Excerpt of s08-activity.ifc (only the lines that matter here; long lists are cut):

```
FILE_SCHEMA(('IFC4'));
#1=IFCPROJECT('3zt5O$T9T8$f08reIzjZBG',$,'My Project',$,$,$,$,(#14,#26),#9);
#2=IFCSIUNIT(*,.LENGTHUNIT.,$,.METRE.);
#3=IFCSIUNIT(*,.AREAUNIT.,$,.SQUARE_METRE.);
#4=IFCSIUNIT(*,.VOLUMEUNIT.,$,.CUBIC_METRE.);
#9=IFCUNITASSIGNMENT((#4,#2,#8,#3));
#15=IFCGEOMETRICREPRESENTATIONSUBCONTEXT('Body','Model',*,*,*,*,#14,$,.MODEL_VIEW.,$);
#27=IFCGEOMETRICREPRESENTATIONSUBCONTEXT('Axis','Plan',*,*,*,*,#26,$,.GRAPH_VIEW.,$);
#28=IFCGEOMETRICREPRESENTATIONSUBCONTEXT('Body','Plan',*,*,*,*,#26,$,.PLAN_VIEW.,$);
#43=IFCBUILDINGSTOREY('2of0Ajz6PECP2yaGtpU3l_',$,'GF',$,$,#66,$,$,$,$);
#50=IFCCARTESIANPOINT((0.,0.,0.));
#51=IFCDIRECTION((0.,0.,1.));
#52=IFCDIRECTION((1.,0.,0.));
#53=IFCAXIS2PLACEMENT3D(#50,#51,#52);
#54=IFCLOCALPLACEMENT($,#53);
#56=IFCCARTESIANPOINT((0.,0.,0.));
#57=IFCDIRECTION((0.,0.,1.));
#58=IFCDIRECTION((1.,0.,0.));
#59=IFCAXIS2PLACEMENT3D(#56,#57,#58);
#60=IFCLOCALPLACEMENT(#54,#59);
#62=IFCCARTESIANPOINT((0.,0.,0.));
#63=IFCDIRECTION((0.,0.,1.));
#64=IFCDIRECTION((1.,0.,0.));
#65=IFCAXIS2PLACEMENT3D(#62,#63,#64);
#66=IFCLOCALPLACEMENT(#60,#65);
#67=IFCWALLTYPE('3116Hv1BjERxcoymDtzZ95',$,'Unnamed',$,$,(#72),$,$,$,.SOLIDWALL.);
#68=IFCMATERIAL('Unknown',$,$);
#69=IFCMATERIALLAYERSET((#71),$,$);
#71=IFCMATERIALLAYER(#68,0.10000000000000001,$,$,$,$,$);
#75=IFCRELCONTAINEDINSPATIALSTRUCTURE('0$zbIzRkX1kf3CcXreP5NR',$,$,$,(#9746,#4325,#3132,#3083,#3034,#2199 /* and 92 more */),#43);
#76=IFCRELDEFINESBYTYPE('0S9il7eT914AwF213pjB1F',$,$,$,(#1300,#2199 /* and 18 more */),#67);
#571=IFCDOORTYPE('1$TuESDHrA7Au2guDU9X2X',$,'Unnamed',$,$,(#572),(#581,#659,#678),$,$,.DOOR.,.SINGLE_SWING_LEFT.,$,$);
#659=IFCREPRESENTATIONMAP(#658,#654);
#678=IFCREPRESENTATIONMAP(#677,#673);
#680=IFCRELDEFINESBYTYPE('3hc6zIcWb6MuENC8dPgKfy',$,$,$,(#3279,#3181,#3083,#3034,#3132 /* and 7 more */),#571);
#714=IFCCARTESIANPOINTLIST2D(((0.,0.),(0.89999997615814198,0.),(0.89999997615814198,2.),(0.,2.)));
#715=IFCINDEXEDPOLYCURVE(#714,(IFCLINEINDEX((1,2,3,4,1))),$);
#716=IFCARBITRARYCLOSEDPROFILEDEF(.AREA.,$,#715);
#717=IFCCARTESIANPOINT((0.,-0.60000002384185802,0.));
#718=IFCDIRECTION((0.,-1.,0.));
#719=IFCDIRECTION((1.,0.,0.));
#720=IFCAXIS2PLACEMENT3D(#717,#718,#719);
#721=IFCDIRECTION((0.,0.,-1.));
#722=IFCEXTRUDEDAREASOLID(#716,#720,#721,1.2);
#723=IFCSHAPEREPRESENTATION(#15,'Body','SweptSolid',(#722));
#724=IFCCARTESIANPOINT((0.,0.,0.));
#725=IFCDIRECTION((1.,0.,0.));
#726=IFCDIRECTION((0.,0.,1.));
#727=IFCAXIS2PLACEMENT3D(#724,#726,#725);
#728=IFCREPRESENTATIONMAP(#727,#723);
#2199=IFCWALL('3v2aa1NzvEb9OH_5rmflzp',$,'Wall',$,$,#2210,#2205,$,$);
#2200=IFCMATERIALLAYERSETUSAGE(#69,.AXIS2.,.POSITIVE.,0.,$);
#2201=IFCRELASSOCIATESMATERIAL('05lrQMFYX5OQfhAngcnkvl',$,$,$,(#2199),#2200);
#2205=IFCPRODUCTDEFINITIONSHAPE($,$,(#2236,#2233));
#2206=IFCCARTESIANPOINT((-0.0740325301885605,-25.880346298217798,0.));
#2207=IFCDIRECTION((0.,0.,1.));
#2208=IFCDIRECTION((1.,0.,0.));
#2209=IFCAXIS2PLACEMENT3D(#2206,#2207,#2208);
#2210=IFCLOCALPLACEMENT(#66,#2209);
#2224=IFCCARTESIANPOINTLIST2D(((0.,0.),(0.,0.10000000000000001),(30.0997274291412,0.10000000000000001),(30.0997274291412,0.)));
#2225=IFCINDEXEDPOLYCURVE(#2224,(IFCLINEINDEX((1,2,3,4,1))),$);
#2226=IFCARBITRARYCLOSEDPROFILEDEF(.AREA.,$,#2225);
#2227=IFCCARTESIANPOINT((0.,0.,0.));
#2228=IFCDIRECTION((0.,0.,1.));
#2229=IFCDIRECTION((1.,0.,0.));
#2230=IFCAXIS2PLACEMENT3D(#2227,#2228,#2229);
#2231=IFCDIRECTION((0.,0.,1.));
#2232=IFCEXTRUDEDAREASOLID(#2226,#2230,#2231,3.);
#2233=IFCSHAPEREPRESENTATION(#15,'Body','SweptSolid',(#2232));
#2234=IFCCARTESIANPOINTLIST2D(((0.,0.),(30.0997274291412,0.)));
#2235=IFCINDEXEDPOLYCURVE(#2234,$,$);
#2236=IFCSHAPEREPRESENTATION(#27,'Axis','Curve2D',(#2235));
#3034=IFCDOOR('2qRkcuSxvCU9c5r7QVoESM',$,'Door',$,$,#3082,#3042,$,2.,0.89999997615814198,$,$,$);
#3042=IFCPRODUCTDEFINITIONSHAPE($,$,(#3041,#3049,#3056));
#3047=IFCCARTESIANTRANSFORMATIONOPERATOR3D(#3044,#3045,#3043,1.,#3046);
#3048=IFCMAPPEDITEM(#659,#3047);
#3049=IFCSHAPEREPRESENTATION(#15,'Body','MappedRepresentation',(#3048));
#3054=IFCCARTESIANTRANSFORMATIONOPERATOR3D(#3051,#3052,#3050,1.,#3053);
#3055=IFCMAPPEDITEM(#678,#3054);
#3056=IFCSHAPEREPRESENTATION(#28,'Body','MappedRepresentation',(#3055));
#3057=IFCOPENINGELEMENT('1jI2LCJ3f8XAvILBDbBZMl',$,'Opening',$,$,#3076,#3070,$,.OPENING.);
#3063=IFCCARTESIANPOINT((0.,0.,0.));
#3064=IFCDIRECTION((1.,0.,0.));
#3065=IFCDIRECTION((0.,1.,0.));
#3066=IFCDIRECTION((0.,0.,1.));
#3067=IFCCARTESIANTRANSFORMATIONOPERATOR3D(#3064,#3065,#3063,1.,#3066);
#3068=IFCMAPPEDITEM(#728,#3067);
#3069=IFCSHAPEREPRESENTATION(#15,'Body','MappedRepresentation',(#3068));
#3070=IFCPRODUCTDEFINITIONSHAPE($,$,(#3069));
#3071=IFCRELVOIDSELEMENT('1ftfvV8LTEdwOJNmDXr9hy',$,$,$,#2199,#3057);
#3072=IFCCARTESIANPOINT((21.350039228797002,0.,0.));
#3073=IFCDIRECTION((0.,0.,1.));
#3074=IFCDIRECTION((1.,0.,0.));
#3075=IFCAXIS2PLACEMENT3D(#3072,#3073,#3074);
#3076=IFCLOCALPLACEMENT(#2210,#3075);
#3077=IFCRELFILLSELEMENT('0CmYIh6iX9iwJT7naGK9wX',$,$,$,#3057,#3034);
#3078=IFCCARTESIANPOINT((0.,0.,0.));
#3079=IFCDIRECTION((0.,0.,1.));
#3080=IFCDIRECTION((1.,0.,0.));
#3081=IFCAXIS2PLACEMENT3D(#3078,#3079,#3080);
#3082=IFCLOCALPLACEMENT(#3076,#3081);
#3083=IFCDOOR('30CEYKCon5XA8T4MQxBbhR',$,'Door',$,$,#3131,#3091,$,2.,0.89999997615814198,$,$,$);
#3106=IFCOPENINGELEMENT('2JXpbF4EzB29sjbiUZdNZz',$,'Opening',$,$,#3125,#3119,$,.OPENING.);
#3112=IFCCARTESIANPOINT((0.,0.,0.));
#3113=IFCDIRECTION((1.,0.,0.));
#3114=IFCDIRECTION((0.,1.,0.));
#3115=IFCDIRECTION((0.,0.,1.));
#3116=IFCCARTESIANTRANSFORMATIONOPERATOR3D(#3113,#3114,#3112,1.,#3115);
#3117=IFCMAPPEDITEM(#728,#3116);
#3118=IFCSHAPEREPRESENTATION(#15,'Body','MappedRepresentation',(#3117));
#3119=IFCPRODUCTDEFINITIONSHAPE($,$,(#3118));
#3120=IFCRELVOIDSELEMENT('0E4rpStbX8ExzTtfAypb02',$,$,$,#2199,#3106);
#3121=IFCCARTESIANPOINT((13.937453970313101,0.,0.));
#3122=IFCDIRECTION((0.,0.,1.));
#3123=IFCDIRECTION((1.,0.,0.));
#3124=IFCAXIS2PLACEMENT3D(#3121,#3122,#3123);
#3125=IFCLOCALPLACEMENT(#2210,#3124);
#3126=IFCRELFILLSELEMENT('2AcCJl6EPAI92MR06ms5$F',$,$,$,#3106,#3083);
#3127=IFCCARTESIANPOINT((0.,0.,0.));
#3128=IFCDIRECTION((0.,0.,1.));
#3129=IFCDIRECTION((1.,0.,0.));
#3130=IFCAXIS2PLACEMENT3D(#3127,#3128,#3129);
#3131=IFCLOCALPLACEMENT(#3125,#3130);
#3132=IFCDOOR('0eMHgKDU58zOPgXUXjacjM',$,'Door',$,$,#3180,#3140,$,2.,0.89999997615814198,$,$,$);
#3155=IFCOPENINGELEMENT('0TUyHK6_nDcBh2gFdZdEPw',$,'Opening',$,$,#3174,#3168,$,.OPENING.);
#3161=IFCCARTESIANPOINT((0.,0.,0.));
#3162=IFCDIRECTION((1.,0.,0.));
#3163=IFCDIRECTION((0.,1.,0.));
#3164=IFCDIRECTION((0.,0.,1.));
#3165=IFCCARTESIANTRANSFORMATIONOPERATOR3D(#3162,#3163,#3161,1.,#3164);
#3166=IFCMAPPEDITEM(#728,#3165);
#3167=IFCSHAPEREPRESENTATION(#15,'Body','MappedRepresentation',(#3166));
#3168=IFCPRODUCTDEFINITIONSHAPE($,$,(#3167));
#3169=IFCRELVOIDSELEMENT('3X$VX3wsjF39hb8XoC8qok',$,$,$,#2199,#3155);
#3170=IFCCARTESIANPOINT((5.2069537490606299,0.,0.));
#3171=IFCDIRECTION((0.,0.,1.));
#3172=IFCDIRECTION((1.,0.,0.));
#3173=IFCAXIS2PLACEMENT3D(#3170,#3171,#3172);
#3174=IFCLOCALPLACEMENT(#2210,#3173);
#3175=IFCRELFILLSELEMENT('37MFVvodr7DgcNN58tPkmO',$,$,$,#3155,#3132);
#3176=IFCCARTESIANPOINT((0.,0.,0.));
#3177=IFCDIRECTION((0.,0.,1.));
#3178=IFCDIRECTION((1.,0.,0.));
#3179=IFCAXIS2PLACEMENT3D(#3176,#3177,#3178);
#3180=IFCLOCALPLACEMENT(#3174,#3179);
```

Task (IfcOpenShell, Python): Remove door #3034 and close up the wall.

```python
import ifcopenshell
import ifcopenshell.api.feature
import ifcopenshell.api.root
import ifcopenshell.geom
import ifcopenshell.util.shape

model = ifcopenshell.open("s08-activity.ifc")
settings = ifcopenshell.geom.settings()


def volume(element):
    """Net volume in cubic metres, openings subtracted."""
    shape = ifcopenshell.geom.create_shape(settings, element)
    return ifcopenshell.util.shape.get_volume(shape.geometry)


door = model.by_guid("2qRkcuSxvCU9c5r7QVoESM")
opening = door.FillsVoids[0].RelatingOpeningElement
wall = opening.VoidsElements[0].RelatingBuildingElement
before = volume(wall)

ifcopenshell.api.root.remove_product(model, product=door)
ifcopenshell.api.feature.remove_feature(model, feature=opening)

after = volume(wall)

print(f"wall volume {before:.3f} -> {after:.3f} m3")

model.write("s08-activity_v2.ifc")
```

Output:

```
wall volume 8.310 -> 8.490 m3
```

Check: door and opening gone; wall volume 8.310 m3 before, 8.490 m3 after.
